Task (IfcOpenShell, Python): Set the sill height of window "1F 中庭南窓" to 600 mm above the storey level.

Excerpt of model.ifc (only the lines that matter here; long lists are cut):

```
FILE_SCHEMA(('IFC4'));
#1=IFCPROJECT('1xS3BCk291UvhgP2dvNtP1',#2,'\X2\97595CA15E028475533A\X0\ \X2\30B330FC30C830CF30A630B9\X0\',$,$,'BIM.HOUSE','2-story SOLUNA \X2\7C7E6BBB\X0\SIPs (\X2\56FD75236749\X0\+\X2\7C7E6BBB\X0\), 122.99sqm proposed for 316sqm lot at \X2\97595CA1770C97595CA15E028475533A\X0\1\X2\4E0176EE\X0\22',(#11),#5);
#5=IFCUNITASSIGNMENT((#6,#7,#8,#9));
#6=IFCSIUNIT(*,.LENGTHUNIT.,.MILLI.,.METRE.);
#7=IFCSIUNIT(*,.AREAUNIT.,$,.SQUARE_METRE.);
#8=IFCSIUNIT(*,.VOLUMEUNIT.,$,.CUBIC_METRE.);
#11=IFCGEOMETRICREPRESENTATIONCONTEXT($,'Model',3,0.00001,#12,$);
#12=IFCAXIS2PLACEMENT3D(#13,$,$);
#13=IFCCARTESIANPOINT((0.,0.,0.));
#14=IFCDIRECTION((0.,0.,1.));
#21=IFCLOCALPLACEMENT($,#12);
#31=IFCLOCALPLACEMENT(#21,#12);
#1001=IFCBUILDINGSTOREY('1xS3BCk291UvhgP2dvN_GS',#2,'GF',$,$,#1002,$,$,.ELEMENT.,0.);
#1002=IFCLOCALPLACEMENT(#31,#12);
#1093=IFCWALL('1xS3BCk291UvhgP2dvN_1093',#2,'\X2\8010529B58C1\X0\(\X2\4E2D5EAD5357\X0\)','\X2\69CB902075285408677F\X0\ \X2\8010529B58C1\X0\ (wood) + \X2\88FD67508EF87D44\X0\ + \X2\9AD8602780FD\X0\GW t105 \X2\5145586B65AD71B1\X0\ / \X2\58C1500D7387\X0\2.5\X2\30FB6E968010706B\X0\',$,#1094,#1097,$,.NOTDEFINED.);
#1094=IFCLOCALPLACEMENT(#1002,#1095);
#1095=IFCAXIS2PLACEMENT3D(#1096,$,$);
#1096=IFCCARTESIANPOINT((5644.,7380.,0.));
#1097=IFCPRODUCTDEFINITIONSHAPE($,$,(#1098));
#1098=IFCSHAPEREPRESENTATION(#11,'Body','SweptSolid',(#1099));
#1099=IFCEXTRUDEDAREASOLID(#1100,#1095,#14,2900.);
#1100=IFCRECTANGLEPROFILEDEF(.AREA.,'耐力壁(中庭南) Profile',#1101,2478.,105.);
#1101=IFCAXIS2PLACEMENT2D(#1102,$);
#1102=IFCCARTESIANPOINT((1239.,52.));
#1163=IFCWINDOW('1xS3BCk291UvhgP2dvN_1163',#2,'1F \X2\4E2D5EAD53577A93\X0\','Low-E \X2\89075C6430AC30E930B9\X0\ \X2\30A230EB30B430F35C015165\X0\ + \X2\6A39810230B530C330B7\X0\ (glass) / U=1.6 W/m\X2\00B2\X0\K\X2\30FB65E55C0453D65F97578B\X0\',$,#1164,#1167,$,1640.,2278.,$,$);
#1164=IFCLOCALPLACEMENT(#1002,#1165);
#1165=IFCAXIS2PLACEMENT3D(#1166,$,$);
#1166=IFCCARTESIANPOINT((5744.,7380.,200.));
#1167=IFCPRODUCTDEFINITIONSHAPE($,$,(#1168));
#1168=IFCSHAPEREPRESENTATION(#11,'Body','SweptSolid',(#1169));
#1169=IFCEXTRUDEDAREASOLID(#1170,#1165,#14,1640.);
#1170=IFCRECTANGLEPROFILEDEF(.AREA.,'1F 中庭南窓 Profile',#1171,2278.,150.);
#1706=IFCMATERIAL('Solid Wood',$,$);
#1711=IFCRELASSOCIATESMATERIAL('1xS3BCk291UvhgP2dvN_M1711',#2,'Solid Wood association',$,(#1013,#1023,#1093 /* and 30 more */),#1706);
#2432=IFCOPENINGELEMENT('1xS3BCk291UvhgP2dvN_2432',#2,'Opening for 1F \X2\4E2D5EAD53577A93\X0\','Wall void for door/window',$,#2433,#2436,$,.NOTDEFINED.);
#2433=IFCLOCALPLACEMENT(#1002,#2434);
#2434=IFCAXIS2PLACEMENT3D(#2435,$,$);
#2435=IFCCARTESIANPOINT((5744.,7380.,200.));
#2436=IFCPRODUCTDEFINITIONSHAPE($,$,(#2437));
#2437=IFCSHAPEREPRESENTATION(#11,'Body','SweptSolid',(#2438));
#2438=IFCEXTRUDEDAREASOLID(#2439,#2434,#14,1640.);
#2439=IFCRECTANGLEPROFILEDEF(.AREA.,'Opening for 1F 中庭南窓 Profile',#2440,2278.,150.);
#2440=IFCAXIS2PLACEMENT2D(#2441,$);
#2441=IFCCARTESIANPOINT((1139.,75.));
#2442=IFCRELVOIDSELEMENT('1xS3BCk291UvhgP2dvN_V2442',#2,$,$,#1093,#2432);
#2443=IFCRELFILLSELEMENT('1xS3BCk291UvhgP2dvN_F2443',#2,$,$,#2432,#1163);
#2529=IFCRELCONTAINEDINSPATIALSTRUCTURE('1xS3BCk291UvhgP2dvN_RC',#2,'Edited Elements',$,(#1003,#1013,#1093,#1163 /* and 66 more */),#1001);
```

```python
import numpy as np
import ifcopenshell
import ifcopenshell.api.geometry
import ifcopenshell.geom
import ifcopenshell.util.element
import ifcopenshell.util.placement
import ifcopenshell.util.shape
import ifcopenshell.util.unit

model = ifcopenshell.open("model.ifc")
unit_scale = ifcopenshell.util.unit.calculate_unit_scale(model)

window = model.by_id(1163)
opening = window.FillsVoids[0].RelatingOpeningElement
storey = ifcopenshell.util.element.get_container(window, ifc_class="IfcBuildingStorey")
level = ifcopenshell.util.placement.get_local_placement(storey.ObjectPlacement)[2, 3]

# The opening's origin need not be at the sill, so measure its lowest point.
shape = ifcopenshell.geom.create_shape(ifcopenshell.geom.settings(), opening)
bottom = ifcopenshell.util.shape.get_shape_bottom_elevation(shape, shape.geometry) / unit_scale
dz = level + 0.6 / unit_scale - bottom

shift = np.array([0.0, 0.0, dz])
# The window is not placed relative to its opening, so move both.
for product in (opening, window):
    matrix = ifcopenshell.util.placement.get_local_placement(product.ObjectPlacement)
    matrix[:3, 3] += shift
    ifcopenshell.api.geometry.edit_object_placement(model, product=product, matrix=matrix, is_si=False)

print(f"moved by {dz * unit_scale:+.3f} m")

model.write("model-out.ifc")
```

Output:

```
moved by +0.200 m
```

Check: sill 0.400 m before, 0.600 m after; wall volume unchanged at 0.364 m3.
